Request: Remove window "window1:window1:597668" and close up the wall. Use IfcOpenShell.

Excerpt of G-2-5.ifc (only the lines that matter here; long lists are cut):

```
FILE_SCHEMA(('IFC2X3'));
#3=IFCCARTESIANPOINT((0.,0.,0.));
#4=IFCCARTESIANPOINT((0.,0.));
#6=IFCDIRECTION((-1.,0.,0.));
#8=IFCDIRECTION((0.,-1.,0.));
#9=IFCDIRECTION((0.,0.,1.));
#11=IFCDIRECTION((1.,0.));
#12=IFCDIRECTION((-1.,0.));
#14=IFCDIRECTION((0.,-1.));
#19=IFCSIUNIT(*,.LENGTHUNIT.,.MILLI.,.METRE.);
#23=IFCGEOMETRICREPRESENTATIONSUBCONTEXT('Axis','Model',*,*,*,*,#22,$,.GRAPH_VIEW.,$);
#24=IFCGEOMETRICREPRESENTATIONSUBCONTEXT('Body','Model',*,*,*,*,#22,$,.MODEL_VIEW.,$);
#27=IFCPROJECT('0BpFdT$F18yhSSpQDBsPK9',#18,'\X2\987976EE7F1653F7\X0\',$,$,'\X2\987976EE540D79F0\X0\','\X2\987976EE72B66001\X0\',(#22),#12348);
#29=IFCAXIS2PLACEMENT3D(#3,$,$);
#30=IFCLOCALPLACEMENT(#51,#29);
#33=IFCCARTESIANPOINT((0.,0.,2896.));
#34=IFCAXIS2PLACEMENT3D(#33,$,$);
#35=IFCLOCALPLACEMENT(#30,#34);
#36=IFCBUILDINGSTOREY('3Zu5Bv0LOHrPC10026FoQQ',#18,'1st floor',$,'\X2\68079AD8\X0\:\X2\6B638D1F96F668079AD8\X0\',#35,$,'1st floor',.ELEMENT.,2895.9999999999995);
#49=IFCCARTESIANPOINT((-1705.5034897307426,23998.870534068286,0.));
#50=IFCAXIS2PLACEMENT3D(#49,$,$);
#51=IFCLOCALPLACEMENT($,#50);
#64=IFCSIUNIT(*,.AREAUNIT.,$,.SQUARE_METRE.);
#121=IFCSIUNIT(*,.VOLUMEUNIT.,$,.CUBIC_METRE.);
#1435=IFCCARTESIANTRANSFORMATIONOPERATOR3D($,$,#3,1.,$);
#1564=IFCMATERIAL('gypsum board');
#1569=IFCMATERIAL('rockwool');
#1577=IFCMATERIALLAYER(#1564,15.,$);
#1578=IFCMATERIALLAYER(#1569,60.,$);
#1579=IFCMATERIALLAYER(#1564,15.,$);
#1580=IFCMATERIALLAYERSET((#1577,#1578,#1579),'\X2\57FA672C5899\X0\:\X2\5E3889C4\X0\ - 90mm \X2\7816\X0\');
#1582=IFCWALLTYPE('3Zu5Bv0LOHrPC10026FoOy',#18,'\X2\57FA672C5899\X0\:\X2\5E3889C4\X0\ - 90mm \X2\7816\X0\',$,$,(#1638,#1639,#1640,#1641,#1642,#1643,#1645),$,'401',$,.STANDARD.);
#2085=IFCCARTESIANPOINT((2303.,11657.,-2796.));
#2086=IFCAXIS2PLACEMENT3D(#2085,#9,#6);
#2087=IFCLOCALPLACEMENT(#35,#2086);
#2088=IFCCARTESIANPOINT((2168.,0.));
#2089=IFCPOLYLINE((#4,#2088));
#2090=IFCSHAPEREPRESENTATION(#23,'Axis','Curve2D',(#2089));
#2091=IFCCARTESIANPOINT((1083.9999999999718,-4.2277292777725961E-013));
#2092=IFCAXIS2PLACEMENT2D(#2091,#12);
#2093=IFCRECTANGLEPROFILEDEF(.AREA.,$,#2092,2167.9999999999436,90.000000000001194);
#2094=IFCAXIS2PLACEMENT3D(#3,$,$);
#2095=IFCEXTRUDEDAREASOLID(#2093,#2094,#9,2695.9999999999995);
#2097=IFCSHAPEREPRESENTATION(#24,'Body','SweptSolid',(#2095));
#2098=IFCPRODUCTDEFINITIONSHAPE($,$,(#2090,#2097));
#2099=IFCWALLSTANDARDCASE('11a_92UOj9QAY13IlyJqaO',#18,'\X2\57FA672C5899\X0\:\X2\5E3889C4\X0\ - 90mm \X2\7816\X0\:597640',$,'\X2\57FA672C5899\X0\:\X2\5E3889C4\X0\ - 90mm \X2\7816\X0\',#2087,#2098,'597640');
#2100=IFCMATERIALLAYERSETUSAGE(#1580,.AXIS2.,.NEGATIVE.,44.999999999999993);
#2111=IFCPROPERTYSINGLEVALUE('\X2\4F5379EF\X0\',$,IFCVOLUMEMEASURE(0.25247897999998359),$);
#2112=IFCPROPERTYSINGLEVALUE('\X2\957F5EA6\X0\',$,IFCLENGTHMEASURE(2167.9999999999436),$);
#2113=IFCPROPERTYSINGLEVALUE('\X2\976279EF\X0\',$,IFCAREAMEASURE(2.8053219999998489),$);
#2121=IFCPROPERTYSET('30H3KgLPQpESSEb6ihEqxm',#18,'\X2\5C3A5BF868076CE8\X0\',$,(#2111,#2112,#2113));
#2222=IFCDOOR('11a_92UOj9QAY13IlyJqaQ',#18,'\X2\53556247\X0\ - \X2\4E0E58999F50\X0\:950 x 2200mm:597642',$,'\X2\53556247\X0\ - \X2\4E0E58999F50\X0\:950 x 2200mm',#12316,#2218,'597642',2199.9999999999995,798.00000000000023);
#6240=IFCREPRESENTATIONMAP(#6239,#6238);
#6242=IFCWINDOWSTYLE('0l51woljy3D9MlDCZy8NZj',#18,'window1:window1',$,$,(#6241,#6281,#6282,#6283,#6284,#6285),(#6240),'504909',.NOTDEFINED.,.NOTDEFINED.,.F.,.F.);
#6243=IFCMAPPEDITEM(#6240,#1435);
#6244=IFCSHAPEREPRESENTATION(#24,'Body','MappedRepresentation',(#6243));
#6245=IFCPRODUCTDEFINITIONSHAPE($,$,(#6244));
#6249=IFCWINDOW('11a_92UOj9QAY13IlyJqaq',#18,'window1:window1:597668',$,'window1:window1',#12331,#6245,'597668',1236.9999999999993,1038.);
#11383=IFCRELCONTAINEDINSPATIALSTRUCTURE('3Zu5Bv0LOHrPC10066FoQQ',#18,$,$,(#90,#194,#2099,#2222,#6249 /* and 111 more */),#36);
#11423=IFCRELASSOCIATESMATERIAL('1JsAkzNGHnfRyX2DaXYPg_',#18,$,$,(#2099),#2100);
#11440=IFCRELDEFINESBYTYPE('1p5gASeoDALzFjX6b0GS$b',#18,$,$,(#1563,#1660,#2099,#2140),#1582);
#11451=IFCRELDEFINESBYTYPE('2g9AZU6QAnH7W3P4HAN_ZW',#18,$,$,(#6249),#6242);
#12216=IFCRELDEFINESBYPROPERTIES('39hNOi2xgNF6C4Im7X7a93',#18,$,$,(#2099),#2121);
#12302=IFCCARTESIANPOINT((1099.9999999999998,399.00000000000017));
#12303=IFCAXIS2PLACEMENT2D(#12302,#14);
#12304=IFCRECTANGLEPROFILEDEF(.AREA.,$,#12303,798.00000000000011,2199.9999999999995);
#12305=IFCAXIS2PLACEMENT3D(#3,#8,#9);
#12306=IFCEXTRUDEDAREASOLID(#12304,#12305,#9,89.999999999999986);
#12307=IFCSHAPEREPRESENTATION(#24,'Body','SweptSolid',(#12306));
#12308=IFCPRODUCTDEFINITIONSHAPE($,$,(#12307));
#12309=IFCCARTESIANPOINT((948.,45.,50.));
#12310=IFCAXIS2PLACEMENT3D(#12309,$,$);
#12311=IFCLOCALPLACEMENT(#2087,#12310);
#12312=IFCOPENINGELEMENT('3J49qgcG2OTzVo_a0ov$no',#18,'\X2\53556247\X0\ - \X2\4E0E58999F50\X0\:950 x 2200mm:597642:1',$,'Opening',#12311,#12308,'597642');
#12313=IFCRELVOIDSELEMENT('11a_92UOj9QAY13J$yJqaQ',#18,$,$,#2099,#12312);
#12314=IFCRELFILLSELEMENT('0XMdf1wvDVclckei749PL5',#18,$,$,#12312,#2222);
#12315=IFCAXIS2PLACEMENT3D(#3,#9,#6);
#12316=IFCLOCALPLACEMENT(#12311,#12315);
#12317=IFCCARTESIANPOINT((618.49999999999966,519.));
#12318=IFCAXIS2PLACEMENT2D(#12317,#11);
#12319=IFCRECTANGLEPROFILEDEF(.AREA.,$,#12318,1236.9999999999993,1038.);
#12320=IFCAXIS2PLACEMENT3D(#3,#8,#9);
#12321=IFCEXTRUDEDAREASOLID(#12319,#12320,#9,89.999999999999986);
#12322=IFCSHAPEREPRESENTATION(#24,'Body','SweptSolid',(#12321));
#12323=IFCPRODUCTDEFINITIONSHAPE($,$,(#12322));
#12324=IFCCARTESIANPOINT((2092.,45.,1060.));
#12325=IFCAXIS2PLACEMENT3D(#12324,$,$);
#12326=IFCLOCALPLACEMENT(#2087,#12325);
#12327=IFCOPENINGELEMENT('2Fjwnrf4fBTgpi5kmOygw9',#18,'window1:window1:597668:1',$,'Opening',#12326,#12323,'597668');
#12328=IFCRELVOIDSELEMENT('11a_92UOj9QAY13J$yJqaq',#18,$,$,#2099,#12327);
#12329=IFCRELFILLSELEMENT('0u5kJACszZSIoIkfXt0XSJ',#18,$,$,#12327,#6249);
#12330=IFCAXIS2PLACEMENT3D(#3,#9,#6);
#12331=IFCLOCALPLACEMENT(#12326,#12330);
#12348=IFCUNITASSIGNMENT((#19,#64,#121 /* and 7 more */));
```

```python
import ifcopenshell
import ifcopenshell.api.feature
import ifcopenshell.api.pset
import ifcopenshell.api.root
import ifcopenshell.geom
import ifcopenshell.util.element
import ifcopenshell.util.shape
import ifcopenshell.util.unit

model = ifcopenshell.open("G-2-5.ifc")
area_scale = ifcopenshell.util.unit.calculate_unit_scale(model, "AREAUNIT")
volume_scale = ifcopenshell.util.unit.calculate_unit_scale(model, "VOLUMEUNIT")
settings = ifcopenshell.geom.settings()


def volume(element):
    """Net volume in cubic metres, openings subtracted."""
    shape = ifcopenshell.geom.create_shape(settings, element)
    return ifcopenshell.util.shape.get_volume(shape.geometry)


window = model.by_guid("11a_92UOj9QAY13IlyJqaq")
opening = window.FillsVoids[0].RelatingOpeningElement
wall = opening.VoidsElements[0].RelatingBuildingElement
before = volume(wall)

ifcopenshell.api.root.remove_product(model, product=window)
ifcopenshell.api.feature.remove_feature(model, feature=opening)

after = volume(wall)
thickness = 0.09  # wall thickness in metres

# Update the wall's stored quantities.
pset = model.by_id(ifcopenshell.util.element.get_pset(wall, "尺寸标注", should_inherit=False)["id"])
ifcopenshell.api.pset.edit_pset(model, pset=pset, properties={
    "体积": model.create_entity("IfcVolumeMeasure", after / volume_scale),
    "面积": model.create_entity("IfcAreaMeasure", after / thickness / area_scale),
})

print(f"wall volume {before:.3f} -> {after:.3f} m3")

model.write("G-2-5_rev.ifc")
```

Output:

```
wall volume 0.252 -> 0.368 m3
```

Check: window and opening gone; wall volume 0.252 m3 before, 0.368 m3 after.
